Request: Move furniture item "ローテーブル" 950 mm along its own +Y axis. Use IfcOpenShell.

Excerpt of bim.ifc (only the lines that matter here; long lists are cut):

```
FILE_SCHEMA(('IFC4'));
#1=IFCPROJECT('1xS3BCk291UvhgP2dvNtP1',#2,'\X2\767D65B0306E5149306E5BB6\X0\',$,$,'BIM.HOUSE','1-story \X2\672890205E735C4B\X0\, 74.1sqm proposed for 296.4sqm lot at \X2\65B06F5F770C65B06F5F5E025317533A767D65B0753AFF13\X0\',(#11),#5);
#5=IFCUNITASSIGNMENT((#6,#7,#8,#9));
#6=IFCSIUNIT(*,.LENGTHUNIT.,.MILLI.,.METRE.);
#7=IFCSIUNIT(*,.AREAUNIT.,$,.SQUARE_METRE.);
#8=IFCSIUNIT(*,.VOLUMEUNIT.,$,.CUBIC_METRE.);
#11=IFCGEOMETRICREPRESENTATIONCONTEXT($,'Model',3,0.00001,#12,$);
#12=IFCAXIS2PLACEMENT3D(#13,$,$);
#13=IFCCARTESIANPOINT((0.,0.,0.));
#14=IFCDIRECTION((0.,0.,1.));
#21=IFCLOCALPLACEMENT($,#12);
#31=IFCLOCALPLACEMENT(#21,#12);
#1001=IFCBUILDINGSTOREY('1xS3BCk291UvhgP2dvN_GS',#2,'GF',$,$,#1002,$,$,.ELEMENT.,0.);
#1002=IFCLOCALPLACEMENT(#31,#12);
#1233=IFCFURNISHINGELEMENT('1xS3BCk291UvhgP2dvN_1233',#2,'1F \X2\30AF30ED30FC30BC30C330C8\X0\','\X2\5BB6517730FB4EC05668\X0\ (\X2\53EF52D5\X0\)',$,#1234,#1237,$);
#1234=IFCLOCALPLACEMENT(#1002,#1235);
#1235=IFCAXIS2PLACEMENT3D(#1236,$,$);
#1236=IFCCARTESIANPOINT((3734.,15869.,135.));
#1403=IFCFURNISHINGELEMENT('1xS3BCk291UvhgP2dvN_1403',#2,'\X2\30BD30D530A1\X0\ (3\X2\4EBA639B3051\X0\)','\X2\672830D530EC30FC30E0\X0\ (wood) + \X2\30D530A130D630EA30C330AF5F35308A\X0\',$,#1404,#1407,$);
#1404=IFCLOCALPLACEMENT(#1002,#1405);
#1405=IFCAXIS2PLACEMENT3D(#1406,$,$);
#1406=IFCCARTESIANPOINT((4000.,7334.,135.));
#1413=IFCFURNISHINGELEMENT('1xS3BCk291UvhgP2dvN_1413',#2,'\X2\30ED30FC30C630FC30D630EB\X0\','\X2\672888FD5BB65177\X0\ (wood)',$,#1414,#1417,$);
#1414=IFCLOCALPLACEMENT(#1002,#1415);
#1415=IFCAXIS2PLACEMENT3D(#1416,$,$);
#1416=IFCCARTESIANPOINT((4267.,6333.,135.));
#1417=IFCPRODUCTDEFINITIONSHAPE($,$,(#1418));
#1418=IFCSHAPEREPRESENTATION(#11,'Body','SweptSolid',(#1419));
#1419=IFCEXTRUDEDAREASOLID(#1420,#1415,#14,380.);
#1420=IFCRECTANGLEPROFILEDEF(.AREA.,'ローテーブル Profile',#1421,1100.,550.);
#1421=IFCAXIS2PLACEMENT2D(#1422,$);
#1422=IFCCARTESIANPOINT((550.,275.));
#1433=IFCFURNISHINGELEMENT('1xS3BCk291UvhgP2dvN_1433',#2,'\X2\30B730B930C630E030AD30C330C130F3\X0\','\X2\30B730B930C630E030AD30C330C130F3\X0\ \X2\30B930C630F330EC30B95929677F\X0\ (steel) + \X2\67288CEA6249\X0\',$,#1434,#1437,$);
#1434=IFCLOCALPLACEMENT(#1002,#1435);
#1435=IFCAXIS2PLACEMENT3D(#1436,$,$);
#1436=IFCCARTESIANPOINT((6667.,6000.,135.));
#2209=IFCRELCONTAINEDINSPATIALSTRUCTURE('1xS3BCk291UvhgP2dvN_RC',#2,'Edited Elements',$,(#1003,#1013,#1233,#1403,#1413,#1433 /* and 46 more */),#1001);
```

```python
import ifcopenshell
import ifcopenshell.api.geometry
import ifcopenshell.util.placement

model = ifcopenshell.open("bim.ifc")

item = model.by_id(1413)
matrix = ifcopenshell.util.placement.get_local_placement(item.ObjectPlacement)
matrix[:3, 3] += matrix[:3, 1] * 950.0
ifcopenshell.api.geometry.edit_object_placement(model, product=item, matrix=matrix, is_si=False)

print(ifcopenshell.util.placement.get_local_placement(item.ObjectPlacement).round(3) + 0.0)

model.write("bim_rev.ifc")
```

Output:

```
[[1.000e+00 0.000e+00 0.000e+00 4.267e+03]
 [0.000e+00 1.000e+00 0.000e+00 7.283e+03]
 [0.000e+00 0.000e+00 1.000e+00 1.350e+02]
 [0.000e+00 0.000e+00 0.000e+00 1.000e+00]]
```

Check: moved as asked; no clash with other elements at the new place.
